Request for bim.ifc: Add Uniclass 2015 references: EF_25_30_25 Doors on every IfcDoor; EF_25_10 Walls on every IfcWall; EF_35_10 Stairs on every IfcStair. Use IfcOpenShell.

First a look at what the model holds.

```python
import ifcopenshell

model = ifcopenshell.open("bim.ifc")
print(model.schema)
print("classifications:", [c.Name for c in model.by_type("IfcClassification")])
for ifc_class in ("IfcDoor", "IfcRoof", "IfcStair", "IfcWall", "IfcWindow"):
    print(ifc_class, len(model.by_type(ifc_class)))
```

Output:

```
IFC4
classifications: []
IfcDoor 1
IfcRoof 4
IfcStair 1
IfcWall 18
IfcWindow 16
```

```python
import ifcopenshell
import ifcopenshell.api.classification

model = ifcopenshell.open("bim.ifc")

system = ifcopenshell.api.classification.add_classification(model, classification="Uniclass 2015")

codes = {
    "IfcDoor": ("EF_25_30_25", "Doors"),
    "IfcWall": ("EF_25_10", "Walls"),
    "IfcStair": ("EF_35_10", "Stairs"),
}
for ifc_class, (code, name) in codes.items():
    products = model.by_type(ifc_class)
    ifcopenshell.api.classification.add_reference(
        model, products=products, classification=system, identification=code, name=name
    )
    print(code, len(products))

model.write("bim_v2.ifc")
```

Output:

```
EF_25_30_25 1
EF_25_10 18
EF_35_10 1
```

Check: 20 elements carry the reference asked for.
